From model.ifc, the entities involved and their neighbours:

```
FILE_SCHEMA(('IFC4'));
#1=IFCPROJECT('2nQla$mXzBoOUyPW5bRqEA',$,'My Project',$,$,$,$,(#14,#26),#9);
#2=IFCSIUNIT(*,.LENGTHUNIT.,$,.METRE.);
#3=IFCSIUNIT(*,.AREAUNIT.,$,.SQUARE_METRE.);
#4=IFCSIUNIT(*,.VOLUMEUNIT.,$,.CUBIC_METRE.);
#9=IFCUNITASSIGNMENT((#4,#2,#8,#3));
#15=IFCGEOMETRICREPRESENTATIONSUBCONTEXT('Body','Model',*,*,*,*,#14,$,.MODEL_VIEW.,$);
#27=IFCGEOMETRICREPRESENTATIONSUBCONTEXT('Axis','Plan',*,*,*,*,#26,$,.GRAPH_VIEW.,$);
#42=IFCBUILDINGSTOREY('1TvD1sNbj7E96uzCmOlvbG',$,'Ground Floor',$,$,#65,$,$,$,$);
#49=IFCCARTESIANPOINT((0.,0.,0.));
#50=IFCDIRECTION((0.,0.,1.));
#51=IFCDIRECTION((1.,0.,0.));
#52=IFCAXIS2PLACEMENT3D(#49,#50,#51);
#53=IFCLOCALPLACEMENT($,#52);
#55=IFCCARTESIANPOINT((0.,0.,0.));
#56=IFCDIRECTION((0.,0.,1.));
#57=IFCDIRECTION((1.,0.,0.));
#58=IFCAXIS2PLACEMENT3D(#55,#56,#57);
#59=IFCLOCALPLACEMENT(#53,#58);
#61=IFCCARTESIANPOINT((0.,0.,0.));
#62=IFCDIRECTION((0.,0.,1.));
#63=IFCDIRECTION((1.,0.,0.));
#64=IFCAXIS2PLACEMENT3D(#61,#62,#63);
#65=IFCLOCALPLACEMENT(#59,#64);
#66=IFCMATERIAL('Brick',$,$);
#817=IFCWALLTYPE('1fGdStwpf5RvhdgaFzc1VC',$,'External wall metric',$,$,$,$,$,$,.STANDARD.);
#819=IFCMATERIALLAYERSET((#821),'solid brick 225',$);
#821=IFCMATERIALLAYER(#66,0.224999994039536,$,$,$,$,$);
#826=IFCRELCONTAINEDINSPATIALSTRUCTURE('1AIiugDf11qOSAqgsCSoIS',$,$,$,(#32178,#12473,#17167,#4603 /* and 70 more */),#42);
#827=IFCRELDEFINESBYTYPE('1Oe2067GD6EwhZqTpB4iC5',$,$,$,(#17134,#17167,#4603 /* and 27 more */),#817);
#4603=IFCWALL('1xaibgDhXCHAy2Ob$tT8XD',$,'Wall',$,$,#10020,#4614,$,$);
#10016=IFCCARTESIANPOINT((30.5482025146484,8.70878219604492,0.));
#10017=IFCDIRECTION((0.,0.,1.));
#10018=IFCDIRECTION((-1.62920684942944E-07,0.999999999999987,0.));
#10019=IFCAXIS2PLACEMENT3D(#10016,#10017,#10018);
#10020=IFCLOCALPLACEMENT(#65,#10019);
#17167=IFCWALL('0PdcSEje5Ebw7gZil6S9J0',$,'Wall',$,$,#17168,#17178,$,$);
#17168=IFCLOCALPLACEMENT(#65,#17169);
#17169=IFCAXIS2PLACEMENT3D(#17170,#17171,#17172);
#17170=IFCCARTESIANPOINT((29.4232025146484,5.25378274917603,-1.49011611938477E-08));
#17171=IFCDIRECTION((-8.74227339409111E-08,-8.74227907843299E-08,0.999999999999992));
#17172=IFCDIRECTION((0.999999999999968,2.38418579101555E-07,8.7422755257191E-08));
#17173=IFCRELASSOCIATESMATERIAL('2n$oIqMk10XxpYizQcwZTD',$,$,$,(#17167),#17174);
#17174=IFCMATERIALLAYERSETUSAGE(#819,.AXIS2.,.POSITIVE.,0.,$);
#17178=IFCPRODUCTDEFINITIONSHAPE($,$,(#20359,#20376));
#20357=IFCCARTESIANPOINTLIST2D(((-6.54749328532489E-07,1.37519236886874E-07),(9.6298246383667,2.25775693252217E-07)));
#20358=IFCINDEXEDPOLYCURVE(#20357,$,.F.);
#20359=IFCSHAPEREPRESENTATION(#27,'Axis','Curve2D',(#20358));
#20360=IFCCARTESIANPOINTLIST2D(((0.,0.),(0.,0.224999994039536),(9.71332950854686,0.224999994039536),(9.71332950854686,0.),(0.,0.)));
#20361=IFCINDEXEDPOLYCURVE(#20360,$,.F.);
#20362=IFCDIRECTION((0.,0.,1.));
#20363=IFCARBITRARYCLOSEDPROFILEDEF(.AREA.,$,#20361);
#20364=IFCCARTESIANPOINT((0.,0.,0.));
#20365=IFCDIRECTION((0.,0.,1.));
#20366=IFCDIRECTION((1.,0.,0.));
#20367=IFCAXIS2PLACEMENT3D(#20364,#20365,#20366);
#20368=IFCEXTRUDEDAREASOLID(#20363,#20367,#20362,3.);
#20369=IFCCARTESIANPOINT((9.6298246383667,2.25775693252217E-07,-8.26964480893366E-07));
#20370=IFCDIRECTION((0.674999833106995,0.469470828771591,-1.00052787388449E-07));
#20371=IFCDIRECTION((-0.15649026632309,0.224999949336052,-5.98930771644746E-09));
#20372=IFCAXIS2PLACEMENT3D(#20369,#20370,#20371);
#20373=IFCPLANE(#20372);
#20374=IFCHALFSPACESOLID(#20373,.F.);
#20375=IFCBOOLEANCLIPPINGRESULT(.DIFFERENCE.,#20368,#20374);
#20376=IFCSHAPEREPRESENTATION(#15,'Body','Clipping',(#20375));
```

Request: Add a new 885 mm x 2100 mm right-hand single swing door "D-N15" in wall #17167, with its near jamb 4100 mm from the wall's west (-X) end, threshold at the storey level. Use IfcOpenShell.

```python
import numpy as np
import ifcopenshell
import ifcopenshell.api.feature
import ifcopenshell.api.geometry
import ifcopenshell.api.root
import ifcopenshell.api.spatial
import ifcopenshell.geom
import ifcopenshell.util.element
import ifcopenshell.util.placement
import ifcopenshell.util.representation
import ifcopenshell.util.shape
import ifcopenshell.util.unit

model = ifcopenshell.open("model.ifc")
unit_scale = ifcopenshell.util.unit.calculate_unit_scale(model)
settings = ifcopenshell.geom.settings()


def volume(element):
    """Net volume in cubic metres, openings subtracted."""
    shape = ifcopenshell.geom.create_shape(settings, element)
    return ifcopenshell.util.shape.get_volume(shape.geometry)


wall = model.by_guid("0PdcSEje5Ebw7gZil6S9J0")
storey = ifcopenshell.util.element.get_container(wall, ifc_class="IfcBuildingStorey")
context = ifcopenshell.util.representation.get_context(model, "Model", "Body", "MODEL_VIEW")
before = volume(wall)

width, height, from_end, sill = 0.885, 2.1, 4.1, 0.0  # metres

# The wall runs along its own X axis, and the end named is its -X end.
wall_shape = ifcopenshell.geom.create_shape(settings, wall)
x, y, z = ifcopenshell.util.shape.get_vertices(wall_shape.geometry).T
start = x.min() + from_end
face, thickness = float(y.min()), float(y.max() - y.min())
wall_matrix = ifcopenshell.util.placement.get_local_placement(wall.ObjectPlacement)
level = ifcopenshell.util.placement.get_local_placement(storey.ObjectPlacement)[2, 3]


def in_wall(x, y):
    """Placement at x, y metres in the wall's axes, at sill height."""
    matrix = wall_matrix.copy()
    matrix[:, 3] = wall_matrix @ np.array([x / unit_scale, y / unit_scale, 0.0, 1.0])
    matrix[2, 3] = level + sill / unit_scale
    return matrix


# Opening: a box that overshoots both wall faces by 50 mm.
opening = ifcopenshell.api.root.create_entity(model, ifc_class="IfcOpeningElement", predefined_type="OPENING")
box = ifcopenshell.api.geometry.add_wall_representation(
    model, context=context, length=width, height=height, thickness=thickness + 0.1
)
ifcopenshell.api.geometry.assign_representation(model, product=opening, representation=box)
ifcopenshell.api.geometry.edit_object_placement(model, product=opening, matrix=in_wall(start, face - 0.05), is_si=False)
ifcopenshell.api.feature.add_feature(model, feature=opening, element=wall)

door = ifcopenshell.api.root.create_entity(model, ifc_class="IfcDoor", name="D-N15", predefined_type="DOOR")
door.OverallWidth, door.OverallHeight = width / unit_scale, height / unit_scale
door.OperationType = "SINGLE_SWING_RIGHT"
body = ifcopenshell.api.geometry.add_door_representation(
    model,
    context=context,
    overall_width=door.OverallWidth,
    overall_height=door.OverallHeight,
    operation_type="SINGLE_SWING_RIGHT",
    lining_properties={"LiningDepth": thickness / unit_scale, "ThresholdDepth": thickness / unit_scale},
)
ifcopenshell.api.geometry.assign_representation(model, product=door, representation=body)
ifcopenshell.api.spatial.assign_container(model, products=[door], relating_structure=storey)
ifcopenshell.api.feature.add_filling(model, opening=opening, element=door)

# The lining spans the wall, so the door starts at the wall face.
ifcopenshell.api.geometry.edit_object_placement(model, product=door, matrix=in_wall(start, face), is_si=False)

after = volume(wall)

print(f"wall volume {before:.3f} -> {after:.3f} m3")

model.write("model_v2.ifc")
```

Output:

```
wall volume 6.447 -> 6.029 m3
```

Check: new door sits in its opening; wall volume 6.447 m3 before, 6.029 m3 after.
